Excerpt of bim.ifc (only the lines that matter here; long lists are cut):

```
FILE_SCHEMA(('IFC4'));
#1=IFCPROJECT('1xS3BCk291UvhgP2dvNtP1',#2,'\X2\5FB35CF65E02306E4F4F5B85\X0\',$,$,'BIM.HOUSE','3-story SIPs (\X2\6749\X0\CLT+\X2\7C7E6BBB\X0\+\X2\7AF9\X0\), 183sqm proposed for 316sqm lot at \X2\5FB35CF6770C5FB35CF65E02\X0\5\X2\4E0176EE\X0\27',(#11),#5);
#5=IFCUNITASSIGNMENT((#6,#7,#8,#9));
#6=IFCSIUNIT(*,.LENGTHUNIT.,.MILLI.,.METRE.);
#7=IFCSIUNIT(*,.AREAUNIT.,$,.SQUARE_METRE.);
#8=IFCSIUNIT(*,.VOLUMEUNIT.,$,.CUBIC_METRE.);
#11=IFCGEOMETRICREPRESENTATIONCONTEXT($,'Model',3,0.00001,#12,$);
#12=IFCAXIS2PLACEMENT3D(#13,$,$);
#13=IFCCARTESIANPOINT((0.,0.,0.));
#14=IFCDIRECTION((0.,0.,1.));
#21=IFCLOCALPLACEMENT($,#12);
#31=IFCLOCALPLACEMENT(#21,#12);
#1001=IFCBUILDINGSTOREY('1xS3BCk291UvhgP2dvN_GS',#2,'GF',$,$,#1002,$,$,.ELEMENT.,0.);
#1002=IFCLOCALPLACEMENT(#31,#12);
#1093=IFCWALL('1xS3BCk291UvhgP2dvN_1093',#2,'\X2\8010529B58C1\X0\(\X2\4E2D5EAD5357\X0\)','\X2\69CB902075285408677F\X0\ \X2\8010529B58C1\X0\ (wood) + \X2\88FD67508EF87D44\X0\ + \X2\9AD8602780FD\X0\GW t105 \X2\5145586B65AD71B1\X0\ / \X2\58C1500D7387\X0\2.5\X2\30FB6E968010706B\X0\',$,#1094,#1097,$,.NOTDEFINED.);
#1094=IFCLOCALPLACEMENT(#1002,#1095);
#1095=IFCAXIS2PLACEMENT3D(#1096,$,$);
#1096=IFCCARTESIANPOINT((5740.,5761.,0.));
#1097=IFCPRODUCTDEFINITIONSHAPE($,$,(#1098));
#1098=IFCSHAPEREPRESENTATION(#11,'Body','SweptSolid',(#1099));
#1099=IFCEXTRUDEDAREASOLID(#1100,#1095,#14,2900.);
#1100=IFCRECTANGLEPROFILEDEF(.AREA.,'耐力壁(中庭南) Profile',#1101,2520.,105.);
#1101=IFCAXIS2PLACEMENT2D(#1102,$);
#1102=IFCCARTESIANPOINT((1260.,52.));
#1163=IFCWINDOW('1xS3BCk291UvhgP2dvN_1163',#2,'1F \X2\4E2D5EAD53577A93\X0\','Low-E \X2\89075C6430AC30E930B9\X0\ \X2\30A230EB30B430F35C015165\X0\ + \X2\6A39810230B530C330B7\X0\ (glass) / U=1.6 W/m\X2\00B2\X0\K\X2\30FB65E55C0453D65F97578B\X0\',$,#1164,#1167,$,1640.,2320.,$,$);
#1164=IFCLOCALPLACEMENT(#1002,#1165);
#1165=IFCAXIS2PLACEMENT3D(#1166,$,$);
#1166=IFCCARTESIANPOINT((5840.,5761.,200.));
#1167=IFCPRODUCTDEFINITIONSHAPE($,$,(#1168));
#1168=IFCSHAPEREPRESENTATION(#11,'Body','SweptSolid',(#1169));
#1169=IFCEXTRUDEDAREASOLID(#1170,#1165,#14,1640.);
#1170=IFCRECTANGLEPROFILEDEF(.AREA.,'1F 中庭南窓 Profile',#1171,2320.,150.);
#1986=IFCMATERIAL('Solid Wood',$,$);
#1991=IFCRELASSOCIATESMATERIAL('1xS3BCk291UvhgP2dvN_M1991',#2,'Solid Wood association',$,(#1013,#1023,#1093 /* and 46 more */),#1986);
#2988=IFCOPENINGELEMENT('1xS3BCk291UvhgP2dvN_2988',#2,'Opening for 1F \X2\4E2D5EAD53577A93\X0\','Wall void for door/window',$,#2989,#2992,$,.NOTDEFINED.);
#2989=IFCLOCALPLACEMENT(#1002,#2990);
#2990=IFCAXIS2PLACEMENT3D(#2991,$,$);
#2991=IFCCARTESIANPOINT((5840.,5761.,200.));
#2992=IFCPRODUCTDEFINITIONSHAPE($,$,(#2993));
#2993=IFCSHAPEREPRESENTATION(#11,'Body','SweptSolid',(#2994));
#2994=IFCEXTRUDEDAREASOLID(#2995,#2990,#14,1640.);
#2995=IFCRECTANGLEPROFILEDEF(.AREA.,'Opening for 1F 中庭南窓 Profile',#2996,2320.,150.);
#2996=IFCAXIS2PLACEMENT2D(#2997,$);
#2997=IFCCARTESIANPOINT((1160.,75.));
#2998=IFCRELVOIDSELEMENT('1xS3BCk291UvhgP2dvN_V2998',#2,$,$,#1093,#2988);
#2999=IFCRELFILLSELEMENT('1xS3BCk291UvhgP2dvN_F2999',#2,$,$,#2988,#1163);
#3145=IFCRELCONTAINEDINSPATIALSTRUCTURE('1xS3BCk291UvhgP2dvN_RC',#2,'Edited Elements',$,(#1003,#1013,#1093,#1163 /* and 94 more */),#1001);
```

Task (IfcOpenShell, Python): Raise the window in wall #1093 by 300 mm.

```python
import numpy as np
import ifcopenshell
import ifcopenshell.api.geometry
import ifcopenshell.util.placement
import ifcopenshell.util.unit

model = ifcopenshell.open("bim.ifc")
unit_scale = ifcopenshell.util.unit.calculate_unit_scale(model)

window = model.by_guid("1xS3BCk291UvhgP2dvN_1163")
opening = window.FillsVoids[0].RelatingOpeningElement
dz = 0.3 / unit_scale

shift = np.array([0.0, 0.0, dz])
# The window is not placed relative to its opening, so move both.
for product in (opening, window):
    matrix = ifcopenshell.util.placement.get_local_placement(product.ObjectPlacement)
    matrix[:3, 3] += shift
    ifcopenshell.api.geometry.edit_object_placement(model, product=product, matrix=matrix, is_si=False)

print(f"moved by {dz * unit_scale:+.3f} m")

model.write("bim-out.ifc")
```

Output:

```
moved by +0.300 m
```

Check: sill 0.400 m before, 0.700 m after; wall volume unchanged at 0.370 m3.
